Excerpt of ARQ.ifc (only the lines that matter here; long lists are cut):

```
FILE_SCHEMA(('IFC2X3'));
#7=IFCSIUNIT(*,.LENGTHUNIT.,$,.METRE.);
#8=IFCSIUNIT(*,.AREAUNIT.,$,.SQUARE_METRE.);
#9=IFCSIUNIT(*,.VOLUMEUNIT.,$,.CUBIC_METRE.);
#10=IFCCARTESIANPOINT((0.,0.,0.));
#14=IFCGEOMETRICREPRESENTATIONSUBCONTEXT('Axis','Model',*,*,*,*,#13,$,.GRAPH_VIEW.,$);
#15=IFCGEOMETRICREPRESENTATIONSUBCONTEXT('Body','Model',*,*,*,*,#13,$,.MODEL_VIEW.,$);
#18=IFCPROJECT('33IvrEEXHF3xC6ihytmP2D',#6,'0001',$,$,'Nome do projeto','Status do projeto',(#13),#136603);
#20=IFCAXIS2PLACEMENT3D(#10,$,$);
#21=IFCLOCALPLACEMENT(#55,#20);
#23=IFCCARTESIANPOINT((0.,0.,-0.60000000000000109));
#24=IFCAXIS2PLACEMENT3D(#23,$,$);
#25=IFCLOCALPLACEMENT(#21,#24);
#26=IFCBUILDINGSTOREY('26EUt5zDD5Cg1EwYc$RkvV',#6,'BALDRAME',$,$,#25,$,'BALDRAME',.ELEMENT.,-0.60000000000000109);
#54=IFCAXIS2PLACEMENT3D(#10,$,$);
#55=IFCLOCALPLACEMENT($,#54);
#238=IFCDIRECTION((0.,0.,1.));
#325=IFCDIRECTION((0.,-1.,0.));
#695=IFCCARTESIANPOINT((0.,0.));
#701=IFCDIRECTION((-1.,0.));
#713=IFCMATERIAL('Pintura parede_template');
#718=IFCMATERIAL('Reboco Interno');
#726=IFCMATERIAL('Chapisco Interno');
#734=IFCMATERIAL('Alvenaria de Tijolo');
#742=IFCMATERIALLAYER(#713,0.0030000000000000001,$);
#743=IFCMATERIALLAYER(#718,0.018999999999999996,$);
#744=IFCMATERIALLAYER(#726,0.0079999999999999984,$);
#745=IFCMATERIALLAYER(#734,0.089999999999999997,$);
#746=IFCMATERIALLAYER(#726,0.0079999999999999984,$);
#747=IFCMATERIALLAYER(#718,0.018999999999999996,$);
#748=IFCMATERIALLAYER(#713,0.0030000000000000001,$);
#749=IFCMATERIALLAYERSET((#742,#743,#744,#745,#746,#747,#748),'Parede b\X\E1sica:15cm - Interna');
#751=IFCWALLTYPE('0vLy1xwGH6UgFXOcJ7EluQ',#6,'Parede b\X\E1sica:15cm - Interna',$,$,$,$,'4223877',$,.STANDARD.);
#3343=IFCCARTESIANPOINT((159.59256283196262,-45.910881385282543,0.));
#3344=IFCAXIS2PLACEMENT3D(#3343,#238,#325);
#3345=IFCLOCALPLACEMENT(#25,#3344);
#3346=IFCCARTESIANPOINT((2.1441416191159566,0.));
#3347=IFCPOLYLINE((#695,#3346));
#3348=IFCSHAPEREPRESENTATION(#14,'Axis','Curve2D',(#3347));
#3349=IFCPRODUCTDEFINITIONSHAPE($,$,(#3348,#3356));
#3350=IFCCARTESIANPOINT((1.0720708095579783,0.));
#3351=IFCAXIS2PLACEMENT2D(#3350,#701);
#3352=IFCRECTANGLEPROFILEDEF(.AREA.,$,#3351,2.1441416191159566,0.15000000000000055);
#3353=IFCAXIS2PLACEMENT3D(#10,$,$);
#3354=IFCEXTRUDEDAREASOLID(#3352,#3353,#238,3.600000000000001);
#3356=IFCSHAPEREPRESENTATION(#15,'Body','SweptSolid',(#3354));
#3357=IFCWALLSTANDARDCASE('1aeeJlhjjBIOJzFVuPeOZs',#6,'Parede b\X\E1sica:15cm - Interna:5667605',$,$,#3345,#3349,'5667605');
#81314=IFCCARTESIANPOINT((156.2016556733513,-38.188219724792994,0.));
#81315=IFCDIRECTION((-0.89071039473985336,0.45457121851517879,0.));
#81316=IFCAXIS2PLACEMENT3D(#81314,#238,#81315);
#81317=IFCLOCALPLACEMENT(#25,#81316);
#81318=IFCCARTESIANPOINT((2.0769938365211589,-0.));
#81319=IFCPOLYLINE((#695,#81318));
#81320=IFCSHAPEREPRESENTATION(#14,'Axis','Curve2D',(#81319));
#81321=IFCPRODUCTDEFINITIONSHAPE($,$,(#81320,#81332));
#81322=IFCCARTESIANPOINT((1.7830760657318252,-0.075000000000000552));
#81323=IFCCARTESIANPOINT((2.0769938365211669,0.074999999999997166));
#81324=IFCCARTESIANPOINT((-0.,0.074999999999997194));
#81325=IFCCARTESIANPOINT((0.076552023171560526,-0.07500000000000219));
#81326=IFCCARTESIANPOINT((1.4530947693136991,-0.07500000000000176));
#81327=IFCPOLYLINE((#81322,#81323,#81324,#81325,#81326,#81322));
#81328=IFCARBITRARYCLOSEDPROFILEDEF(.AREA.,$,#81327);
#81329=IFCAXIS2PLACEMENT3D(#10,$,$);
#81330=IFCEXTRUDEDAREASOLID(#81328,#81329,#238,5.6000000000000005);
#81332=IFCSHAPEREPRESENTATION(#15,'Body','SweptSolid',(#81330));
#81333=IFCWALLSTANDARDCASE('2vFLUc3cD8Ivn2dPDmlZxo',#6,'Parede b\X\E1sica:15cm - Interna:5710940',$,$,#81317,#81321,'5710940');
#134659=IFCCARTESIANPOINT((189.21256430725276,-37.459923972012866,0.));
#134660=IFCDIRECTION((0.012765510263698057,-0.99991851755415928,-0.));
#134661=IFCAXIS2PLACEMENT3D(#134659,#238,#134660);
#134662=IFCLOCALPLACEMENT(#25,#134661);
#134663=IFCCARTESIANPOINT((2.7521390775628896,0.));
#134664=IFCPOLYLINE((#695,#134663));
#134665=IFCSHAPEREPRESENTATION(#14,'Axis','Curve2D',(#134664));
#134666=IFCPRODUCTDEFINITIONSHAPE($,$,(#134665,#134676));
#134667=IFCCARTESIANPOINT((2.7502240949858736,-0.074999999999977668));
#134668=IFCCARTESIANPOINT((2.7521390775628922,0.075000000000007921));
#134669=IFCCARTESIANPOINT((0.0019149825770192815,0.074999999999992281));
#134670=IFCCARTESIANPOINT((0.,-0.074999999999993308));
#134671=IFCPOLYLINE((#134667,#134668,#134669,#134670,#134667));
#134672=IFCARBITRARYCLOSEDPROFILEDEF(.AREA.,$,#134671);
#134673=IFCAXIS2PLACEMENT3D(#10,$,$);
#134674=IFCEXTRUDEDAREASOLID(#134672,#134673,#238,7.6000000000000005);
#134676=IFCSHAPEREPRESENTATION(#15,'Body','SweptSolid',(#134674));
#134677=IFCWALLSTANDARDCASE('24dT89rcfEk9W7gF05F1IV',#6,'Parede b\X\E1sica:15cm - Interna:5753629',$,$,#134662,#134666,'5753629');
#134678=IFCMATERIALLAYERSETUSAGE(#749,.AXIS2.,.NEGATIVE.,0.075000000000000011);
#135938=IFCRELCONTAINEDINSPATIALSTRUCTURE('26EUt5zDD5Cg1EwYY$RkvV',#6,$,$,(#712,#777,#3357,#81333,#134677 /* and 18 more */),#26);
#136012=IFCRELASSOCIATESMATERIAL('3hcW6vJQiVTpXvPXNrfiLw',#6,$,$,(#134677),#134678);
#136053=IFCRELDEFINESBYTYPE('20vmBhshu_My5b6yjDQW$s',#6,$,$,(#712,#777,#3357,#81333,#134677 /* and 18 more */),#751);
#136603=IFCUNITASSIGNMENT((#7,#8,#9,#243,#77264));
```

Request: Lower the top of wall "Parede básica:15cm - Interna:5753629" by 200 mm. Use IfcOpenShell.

```python
import ifcopenshell
import ifcopenshell.geom
import ifcopenshell.util.representation
import ifcopenshell.util.shape

model = ifcopenshell.open("ARQ.ifc")
settings = ifcopenshell.geom.settings()


def volume(element):
    """Net volume in cubic metres, openings subtracted."""
    shape = ifcopenshell.geom.create_shape(settings, element)
    return ifcopenshell.util.shape.get_volume(shape.geometry)


wall = model.by_id(134677)
before = volume(wall)

body = ifcopenshell.util.representation.get_representation(wall, "Model", "Body")
solid = body.Items[0]
old_height = solid.Depth
solid.Depth -= 0.2
after = volume(wall)

print(f"height {old_height:g} -> {solid.Depth:g}, volume {before:.3f} -> {after:.3f} m3")

model.write("ARQ_v2.ifc")
```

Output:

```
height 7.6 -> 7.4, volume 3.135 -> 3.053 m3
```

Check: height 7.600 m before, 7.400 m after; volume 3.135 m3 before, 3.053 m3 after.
